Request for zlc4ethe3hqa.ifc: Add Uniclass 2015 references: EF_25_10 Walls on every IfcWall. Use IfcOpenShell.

First a look at what the model holds.

```python
import ifcopenshell

model = ifcopenshell.open("zlc4ethe3hqa.ifc")
print(model.schema)
print("classifications:", [c.Name for c in model.by_type("IfcClassification")])
for ifc_class in ("IfcDoor", "IfcRoof", "IfcStair", "IfcWall", "IfcWindow"):
    print(ifc_class, len(model.by_type(ifc_class)))
```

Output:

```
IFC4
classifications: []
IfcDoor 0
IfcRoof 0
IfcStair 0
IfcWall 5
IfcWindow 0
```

```python
import ifcopenshell
import ifcopenshell.api.classification

model = ifcopenshell.open("zlc4ethe3hqa.ifc")

system = ifcopenshell.api.classification.add_classification(model, classification="Uniclass 2015")

codes = {
    "IfcWall": ("EF_25_10", "Walls"),
}
for ifc_class, (code, name) in codes.items():
    products = model.by_type(ifc_class)
    ifcopenshell.api.classification.add_reference(
        model, products=products, classification=system, identification=code, name=name
    )
    print(code, len(products))

model.write("zlc4ethe3hqa_rev.ifc")
```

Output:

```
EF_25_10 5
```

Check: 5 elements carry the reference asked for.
